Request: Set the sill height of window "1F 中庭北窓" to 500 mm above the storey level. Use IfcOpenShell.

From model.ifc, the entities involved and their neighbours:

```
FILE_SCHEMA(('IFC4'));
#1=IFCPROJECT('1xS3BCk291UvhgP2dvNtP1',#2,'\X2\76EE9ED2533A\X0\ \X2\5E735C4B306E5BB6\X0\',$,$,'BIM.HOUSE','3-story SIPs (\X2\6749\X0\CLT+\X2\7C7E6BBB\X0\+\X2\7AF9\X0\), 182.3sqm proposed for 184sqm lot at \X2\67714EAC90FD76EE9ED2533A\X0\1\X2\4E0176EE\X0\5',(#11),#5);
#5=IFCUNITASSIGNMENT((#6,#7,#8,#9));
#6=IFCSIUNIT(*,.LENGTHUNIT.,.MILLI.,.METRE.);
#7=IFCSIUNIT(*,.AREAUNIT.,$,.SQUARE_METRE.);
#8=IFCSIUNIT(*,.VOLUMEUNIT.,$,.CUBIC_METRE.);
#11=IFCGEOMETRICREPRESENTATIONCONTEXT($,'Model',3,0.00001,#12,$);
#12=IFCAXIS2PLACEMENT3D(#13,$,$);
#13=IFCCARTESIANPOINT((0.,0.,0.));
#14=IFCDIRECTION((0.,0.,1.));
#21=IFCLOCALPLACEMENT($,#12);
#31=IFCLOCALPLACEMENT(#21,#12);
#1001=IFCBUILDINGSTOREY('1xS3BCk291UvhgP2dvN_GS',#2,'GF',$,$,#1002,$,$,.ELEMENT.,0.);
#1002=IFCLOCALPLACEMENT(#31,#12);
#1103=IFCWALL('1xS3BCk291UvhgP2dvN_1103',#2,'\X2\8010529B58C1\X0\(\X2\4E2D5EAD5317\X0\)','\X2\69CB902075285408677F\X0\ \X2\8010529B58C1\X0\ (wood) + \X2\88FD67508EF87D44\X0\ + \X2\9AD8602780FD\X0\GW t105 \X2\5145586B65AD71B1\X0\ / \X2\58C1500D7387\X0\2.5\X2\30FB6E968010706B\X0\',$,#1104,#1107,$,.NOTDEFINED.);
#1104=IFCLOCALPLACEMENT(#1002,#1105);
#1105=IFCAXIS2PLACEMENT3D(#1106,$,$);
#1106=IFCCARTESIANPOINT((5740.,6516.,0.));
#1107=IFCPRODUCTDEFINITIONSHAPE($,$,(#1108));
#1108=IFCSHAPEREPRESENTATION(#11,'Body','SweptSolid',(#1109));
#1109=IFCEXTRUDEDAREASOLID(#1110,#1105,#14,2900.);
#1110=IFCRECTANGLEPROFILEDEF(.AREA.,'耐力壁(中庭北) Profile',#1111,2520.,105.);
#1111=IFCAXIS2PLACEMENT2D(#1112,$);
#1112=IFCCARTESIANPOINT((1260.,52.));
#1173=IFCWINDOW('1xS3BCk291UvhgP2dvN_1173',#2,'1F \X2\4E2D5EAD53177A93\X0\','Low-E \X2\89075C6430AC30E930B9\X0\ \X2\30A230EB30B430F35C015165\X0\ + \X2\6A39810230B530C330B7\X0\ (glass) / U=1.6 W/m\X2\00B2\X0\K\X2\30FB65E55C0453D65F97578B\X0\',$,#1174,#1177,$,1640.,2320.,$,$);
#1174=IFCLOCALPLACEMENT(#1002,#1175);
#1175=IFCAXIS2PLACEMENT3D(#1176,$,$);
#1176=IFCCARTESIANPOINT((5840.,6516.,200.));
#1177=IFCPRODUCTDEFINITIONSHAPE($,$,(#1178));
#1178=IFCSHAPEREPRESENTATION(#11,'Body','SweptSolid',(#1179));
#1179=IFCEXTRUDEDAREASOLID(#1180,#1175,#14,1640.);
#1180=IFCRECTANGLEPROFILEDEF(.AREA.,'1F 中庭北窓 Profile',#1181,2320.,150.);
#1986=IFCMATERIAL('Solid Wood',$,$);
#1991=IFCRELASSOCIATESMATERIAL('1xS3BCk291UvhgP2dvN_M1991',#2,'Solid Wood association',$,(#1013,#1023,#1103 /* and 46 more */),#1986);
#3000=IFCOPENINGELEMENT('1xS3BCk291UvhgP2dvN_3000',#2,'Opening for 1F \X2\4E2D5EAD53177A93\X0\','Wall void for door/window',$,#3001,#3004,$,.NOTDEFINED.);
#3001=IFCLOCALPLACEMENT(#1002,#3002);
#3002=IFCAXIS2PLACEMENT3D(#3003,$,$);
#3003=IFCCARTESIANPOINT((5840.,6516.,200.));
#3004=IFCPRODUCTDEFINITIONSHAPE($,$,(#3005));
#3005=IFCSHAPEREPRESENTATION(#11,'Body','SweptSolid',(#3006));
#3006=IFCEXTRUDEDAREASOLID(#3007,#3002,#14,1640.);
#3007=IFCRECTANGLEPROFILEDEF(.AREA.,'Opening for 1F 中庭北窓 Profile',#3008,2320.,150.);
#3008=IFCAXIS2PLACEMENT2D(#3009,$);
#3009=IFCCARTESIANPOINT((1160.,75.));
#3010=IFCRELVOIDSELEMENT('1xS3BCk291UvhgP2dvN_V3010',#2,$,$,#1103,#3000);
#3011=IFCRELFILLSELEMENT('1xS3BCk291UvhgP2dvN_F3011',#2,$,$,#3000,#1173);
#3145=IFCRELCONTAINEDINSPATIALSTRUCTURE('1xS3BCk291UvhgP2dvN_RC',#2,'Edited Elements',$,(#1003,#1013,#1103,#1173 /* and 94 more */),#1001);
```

```python
import numpy as np
import ifcopenshell
import ifcopenshell.api.geometry
import ifcopenshell.geom
import ifcopenshell.util.element
import ifcopenshell.util.placement
import ifcopenshell.util.shape
import ifcopenshell.util.unit

model = ifcopenshell.open("model.ifc")
unit_scale = ifcopenshell.util.unit.calculate_unit_scale(model)

window = model.by_guid("1xS3BCk291UvhgP2dvN_1173")
opening = window.FillsVoids[0].RelatingOpeningElement
storey = ifcopenshell.util.element.get_container(window, ifc_class="IfcBuildingStorey")
level = ifcopenshell.util.placement.get_local_placement(storey.ObjectPlacement)[2, 3]

# The opening's origin need not be at the sill, so measure its lowest point.
shape = ifcopenshell.geom.create_shape(ifcopenshell.geom.settings(), opening)
bottom = ifcopenshell.util.shape.get_shape_bottom_elevation(shape, shape.geometry) / unit_scale
dz = level + 0.5 / unit_scale - bottom

shift = np.array([0.0, 0.0, dz])
# The window is not placed relative to its opening, so move both.
for product in (opening, window):
    matrix = ifcopenshell.util.placement.get_local_placement(product.ObjectPlacement)
    matrix[:3, 3] += shift
    ifcopenshell.api.geometry.edit_object_placement(model, product=product, matrix=matrix, is_si=False)

print(f"moved by {dz * unit_scale:+.3f} m")

model.write("model_v2.ifc")
```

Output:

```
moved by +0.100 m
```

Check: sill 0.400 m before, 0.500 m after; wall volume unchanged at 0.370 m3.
